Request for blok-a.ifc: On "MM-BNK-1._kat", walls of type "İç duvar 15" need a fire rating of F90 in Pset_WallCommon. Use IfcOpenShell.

First a look at what the model holds.

```python
import ifcopenshell
import ifcopenshell.util.element

model = ifcopenshell.open("blok-a.ifc")
print(model.schema)
storey = next(s for s in model.by_type("IfcBuildingStorey") if s.Name == "MM-BNK-1._kat")
walls = [e for e in ifcopenshell.util.element.get_decomposition(storey) if e.is_a("IfcWall")]
seen = {}
for e in walls:
    element_type = ifcopenshell.util.element.get_type(e)
    key = (element_type.Name if element_type != e and element_type else None, ifcopenshell.util.element.get_pset(e, "Pset_WallCommon", "FireRating"))
    seen[key] = seen.get(key, 0) + 1
for (name, value), count in sorted(seen.items(), key=str):
    print(count, "x", name, "|", value)
```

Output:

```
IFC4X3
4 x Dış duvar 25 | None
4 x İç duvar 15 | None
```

```python
import ifcopenshell
import ifcopenshell.api.pset
import ifcopenshell.util.element

model = ifcopenshell.open("blok-a.ifc")

storey = next(s for s in model.by_type("IfcBuildingStorey") if s.Name == "MM-BNK-1._kat")
walls = [e for e in ifcopenshell.util.element.get_decomposition(storey) if e.is_a("IfcWall")]

count = 0
for e in walls:
    element_type = ifcopenshell.util.element.get_type(e)
    if element_type in (None, e) or element_type.Name != "İç duvar 15":
        continue
    # add_pset returns the element's existing set when there is one.
    pset = ifcopenshell.api.pset.add_pset(model, product=e, name="Pset_WallCommon")
    ifcopenshell.api.pset.edit_pset(model, pset=pset, properties={"FireRating": "F90"})
    count += 1

print(count, "walls updated")

model.write("blok-a_rev.ifc")
```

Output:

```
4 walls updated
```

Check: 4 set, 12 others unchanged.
